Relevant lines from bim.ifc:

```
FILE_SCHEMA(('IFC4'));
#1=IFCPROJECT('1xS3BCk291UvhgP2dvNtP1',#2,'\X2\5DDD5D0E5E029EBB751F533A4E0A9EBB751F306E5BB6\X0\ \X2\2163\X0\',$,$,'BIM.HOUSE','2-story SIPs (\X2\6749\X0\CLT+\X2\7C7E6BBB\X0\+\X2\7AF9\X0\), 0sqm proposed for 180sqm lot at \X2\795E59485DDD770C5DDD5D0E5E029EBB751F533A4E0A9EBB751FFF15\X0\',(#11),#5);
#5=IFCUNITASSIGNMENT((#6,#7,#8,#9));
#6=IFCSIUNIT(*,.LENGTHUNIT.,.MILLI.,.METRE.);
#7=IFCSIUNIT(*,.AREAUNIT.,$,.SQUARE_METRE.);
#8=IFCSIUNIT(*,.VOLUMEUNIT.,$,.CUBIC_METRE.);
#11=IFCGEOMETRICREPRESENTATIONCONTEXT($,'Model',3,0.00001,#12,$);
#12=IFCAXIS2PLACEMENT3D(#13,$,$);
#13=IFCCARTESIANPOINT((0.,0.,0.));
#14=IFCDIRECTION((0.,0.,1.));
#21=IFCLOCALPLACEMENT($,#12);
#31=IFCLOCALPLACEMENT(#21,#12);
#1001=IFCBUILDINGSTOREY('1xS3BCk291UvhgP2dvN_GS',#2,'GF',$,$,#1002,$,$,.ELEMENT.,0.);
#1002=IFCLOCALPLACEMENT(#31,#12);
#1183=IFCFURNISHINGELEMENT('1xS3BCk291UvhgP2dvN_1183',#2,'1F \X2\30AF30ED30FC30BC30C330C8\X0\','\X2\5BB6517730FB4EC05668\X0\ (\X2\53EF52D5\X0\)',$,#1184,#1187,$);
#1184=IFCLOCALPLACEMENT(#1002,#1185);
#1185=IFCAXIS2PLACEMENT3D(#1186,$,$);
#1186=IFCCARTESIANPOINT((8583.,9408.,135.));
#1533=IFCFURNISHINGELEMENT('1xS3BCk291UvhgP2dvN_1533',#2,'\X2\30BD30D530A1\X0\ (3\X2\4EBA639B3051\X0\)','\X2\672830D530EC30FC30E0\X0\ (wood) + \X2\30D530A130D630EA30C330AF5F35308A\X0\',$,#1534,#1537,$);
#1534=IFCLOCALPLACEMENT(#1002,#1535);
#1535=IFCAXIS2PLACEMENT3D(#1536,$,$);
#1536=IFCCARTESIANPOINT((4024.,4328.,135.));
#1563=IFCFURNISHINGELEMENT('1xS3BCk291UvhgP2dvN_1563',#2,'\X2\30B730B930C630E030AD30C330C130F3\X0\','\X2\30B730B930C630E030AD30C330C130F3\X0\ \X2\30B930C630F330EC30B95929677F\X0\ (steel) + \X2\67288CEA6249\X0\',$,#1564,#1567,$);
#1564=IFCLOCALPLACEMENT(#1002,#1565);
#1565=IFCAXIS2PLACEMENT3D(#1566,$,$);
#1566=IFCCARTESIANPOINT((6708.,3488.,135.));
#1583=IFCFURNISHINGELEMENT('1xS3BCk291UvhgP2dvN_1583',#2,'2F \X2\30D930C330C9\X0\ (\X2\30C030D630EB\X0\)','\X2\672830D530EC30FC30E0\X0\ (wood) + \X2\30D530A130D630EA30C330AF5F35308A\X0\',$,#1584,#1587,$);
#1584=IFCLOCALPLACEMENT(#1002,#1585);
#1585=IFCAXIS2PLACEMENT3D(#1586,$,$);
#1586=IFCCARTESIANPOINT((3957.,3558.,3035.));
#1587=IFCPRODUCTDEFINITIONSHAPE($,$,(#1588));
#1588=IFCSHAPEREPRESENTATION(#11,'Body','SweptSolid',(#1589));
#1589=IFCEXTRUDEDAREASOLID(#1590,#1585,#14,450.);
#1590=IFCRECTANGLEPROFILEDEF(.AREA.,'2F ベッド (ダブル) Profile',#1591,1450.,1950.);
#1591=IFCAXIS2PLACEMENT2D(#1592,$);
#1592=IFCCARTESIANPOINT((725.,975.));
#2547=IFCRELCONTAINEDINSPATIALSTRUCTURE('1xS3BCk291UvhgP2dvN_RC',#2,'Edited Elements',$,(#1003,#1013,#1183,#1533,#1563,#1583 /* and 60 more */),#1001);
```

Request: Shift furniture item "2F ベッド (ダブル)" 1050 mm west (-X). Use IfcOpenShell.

```python
import ifcopenshell
import ifcopenshell.api.geometry
import ifcopenshell.util.placement
import ifcopenshell.util.unit

model = ifcopenshell.open("bim.ifc")
unit_scale = ifcopenshell.util.unit.calculate_unit_scale(model)

item = model.by_guid("1xS3BCk291UvhgP2dvN_1583")
matrix = ifcopenshell.util.placement.get_local_placement(item.ObjectPlacement)
matrix[0, 3] -= 1.05 / unit_scale
ifcopenshell.api.geometry.edit_object_placement(model, product=item, matrix=matrix, is_si=False)

print(ifcopenshell.util.placement.get_local_placement(item.ObjectPlacement).round(3) + 0.0)

model.write("bim_updated.ifc")
```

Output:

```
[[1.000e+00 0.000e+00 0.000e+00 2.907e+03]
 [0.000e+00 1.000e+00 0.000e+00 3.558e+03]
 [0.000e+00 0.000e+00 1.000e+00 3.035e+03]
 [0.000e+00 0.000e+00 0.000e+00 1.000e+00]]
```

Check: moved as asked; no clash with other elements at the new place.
